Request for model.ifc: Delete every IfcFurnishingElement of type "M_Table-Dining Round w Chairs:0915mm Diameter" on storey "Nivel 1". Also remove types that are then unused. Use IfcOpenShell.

First a look at what the model holds.

```python
import ifcopenshell
import ifcopenshell.util.element

model = ifcopenshell.open("model.ifc")
print(model.schema)
storey = next(s for s in model.by_type("IfcBuildingStorey") if s.Name == "Nivel 1")
furniture = [e for e in ifcopenshell.util.element.get_decomposition(storey) if e.is_a("IfcFurnishingElement")]
seen = {}
for e in furniture:
    element_type = ifcopenshell.util.element.get_type(e)
    name = element_type.Name if element_type not in (None, e) else None
    seen[name] = seen.get(name, 0) + 1
for name, count in sorted(seen.items(), key=str):
    print(count, "x", name)
```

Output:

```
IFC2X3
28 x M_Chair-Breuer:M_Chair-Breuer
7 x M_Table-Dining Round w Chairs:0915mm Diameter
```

```python
import ifcopenshell
import ifcopenshell.api.root
import ifcopenshell.util.element

model = ifcopenshell.open("model.ifc")

storey = next(s for s in model.by_type("IfcBuildingStorey") if s.Name == "Nivel 1")
furniture = [e for e in ifcopenshell.util.element.get_decomposition(storey) if e.is_a("IfcFurnishingElement")]
targets = [e for e in furniture if (t := ifcopenshell.util.element.get_type(e)) not in (None, e) and t.Name == "M_Table-Dining Round w Chairs:0915mm Diameter"]
types = {ifcopenshell.util.element.get_type(e) for e in targets} - {None, *targets}

for e in targets:
    ifcopenshell.api.root.remove_product(model, product=e)
print(len(targets), "removed")

unused = [t for t in types if not ifcopenshell.util.element.get_types(t)]
for t in unused:
    ifcopenshell.api.root.remove_product(model, product=t)
print(len(unused), "unused types removed")

model.write("model_rev.ifc")
```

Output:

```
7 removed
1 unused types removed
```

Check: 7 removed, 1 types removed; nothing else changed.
